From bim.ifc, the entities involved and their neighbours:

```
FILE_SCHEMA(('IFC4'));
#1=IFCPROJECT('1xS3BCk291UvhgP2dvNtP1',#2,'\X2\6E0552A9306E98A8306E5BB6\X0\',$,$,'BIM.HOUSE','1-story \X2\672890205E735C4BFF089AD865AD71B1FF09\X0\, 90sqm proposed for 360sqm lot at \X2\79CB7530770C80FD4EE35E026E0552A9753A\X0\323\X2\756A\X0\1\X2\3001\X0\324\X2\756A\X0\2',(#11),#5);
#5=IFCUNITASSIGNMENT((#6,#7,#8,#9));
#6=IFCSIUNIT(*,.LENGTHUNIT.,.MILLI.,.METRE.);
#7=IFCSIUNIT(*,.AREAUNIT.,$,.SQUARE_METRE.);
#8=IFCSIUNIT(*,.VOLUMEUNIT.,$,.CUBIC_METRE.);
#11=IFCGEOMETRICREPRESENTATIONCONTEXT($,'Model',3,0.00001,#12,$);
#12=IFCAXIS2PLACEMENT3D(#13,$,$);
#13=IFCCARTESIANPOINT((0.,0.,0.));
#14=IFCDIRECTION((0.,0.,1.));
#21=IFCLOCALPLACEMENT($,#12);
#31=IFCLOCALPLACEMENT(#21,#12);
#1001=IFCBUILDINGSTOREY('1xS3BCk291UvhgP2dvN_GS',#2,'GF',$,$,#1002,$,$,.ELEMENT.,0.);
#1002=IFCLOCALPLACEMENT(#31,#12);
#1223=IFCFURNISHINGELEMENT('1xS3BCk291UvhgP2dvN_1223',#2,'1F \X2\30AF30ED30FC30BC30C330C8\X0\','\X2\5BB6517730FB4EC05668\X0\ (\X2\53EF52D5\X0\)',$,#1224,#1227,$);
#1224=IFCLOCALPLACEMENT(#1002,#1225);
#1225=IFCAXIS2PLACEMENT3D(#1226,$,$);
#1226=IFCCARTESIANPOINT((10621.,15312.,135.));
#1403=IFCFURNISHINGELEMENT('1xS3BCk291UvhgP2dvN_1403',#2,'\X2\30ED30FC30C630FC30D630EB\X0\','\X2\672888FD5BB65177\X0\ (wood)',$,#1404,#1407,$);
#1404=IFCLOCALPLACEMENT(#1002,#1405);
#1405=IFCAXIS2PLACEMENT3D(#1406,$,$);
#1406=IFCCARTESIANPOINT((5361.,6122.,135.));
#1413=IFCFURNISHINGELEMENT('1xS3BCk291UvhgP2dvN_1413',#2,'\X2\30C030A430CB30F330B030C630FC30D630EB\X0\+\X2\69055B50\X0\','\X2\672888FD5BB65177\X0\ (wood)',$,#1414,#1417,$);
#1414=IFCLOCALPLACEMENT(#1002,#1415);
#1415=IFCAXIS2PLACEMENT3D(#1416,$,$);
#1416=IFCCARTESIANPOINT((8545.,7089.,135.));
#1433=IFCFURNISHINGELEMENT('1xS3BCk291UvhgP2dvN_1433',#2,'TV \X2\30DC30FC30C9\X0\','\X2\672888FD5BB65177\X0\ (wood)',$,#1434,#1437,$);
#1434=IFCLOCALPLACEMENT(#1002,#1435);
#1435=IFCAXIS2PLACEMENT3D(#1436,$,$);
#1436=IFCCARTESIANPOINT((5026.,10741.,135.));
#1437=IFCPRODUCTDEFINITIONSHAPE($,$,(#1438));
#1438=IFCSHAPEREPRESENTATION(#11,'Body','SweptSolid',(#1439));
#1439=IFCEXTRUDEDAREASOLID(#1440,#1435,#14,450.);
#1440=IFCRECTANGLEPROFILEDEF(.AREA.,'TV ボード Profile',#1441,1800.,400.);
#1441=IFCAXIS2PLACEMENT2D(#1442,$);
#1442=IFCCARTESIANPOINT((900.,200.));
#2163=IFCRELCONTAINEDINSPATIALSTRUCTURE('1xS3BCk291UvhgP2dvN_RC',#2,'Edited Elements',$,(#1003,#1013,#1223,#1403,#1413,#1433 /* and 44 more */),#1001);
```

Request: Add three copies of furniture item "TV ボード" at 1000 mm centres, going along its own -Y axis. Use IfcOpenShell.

```python
import ifcopenshell
import ifcopenshell.api.geometry
import ifcopenshell.api.root
import ifcopenshell.util.element
import ifcopenshell.util.placement

model = ifcopenshell.open("bim.ifc")


def reuse_history(source, copy):
    """copy_class also copies each property set's owner history, people and application; keep the originals."""
    for rel in copy.IsDefinedBy:
        if rel.is_a("IfcRelDefinesByProperties") and (history := rel.RelatingPropertyDefinition.OwnerHistory):
            rel.RelatingPropertyDefinition.OwnerHistory = source.OwnerHistory
            ifcopenshell.util.element.remove_deep2(model, history)


source = model.by_id(1433)
base = ifcopenshell.util.placement.get_local_placement(source.ObjectPlacement)
step = -base[:3, 1] * 1000.0

for i in range(1, 4):
    copy = ifcopenshell.api.root.copy_class(model, product=source)
    copy.Representation = ifcopenshell.util.element.copy_deep(
        model, source.Representation, exclude=["IfcGeometricRepresentationContext", "IfcRepresentationMap"]
    )
    reuse_history(source, copy)
    matrix = base.copy()
    matrix[:3, 3] += i * step
    print("added at", matrix[:3, 3].round(3) + 0.0)
    ifcopenshell.api.geometry.edit_object_placement(model, product=copy, matrix=matrix, is_si=False)

model.write("bim_edited.ifc")
```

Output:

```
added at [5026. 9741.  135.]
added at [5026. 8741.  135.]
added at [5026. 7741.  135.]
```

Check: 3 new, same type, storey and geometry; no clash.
